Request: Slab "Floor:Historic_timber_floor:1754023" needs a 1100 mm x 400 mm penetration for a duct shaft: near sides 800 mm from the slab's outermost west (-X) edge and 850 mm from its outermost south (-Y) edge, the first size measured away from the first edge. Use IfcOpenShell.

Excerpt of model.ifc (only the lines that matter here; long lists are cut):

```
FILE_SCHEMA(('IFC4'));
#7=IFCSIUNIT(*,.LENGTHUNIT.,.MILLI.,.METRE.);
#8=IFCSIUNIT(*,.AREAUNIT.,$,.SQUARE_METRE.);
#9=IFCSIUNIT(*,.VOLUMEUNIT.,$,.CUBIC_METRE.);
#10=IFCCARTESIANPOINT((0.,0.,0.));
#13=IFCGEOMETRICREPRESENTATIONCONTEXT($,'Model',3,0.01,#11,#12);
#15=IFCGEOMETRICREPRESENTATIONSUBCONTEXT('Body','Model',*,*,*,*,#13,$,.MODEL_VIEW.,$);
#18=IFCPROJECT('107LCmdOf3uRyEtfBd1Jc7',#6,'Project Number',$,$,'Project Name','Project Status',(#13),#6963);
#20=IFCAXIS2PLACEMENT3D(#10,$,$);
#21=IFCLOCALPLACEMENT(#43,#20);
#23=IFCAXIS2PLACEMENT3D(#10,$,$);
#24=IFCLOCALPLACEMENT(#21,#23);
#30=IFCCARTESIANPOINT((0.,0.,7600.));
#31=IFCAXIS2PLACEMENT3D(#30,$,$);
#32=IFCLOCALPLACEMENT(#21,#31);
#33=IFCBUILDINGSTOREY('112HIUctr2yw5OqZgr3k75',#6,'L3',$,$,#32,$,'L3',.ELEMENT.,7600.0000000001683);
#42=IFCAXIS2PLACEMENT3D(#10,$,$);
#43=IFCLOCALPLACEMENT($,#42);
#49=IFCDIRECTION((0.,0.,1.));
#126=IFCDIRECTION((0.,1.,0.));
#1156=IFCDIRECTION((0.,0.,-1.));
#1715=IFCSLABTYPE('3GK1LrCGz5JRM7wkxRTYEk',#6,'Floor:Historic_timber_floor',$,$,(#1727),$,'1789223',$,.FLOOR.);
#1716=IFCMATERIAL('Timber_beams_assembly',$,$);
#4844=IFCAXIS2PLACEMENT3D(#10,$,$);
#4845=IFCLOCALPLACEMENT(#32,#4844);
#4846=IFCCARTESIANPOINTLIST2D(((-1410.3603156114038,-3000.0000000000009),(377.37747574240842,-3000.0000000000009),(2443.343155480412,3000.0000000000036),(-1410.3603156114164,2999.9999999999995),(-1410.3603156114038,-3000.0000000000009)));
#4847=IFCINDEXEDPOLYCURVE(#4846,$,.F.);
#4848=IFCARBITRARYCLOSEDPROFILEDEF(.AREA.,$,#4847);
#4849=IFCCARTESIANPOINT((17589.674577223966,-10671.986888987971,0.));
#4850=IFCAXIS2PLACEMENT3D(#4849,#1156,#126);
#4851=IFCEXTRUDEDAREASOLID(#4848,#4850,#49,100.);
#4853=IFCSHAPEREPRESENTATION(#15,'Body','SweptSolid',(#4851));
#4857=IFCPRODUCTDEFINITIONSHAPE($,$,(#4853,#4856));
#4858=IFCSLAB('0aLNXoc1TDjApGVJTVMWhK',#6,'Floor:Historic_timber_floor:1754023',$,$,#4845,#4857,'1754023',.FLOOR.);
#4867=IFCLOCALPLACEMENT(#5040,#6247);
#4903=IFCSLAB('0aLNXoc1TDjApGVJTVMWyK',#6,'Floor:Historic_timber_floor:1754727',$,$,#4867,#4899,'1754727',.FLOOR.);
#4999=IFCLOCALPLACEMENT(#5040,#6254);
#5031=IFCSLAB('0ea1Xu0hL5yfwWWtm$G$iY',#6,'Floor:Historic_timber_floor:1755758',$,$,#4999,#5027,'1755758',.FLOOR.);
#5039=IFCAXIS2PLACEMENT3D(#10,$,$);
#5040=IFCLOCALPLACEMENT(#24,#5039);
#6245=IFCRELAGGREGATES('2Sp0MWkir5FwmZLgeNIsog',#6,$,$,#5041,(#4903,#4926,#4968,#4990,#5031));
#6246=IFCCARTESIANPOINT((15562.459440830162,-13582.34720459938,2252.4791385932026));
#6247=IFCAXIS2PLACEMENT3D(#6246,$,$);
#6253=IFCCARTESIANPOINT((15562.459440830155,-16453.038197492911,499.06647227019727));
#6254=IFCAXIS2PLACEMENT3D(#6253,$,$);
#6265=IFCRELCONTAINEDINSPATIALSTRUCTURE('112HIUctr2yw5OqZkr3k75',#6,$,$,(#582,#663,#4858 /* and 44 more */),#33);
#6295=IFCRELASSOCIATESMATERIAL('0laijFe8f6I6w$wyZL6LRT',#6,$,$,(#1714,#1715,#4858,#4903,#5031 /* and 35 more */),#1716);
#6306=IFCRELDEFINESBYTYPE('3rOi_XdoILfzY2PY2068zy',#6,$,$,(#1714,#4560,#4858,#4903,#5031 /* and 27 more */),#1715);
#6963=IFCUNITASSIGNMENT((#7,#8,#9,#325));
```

```python
import numpy as np
import ifcopenshell
import ifcopenshell.api.feature
import ifcopenshell.api.geometry
import ifcopenshell.api.root
import ifcopenshell.geom
import ifcopenshell.util.placement
import ifcopenshell.util.representation
import ifcopenshell.util.shape
import ifcopenshell.util.unit

model = ifcopenshell.open("model.ifc")
unit_scale = ifcopenshell.util.unit.calculate_unit_scale(model)
settings = ifcopenshell.geom.settings()


def volume(element):
    """Net volume in cubic metres, openings subtracted."""
    shape = ifcopenshell.geom.create_shape(settings, element)
    return ifcopenshell.util.shape.get_volume(shape.geometry)


slab = model.by_id(4858)
before = volume(slab)

# Extent in the slab's own axes, in metres. The edges named are its -X and -Y sides.
slab_shape = ifcopenshell.geom.create_shape(settings, slab)
vertices = ifcopenshell.util.shape.get_vertices(slab_shape.geometry)
x_min, y_min, bottom = vertices.min(axis=0)
top = vertices[:, 2].max()

opening = ifcopenshell.api.root.create_entity(model, ifc_class="IfcOpeningElement", name="Duct shaft opening", predefined_type="OPENING")
context = ifcopenshell.util.representation.get_context(model, "Model", "Body", "MODEL_VIEW")
width, depth = 1.1, 0.4
outline = [(0.0, 0.0), (width, 0.0), (width, depth), (0.0, depth), (0.0, 0.0)]
# Overshoot both faces by 50 mm so the cut is clean.
shape = ifcopenshell.api.geometry.add_slab_representation(
    model, context=context, depth=top - bottom + 0.1, polyline=outline
)
ifcopenshell.api.geometry.assign_representation(model, product=opening, representation=shape)

matrix = ifcopenshell.util.placement.get_local_placement(slab.ObjectPlacement)
matrix[:, 3] = matrix @ np.append(np.array([x_min + 0.8, y_min + 0.85, bottom - 0.05]) / unit_scale, 1.0)
ifcopenshell.api.geometry.edit_object_placement(model, product=opening, matrix=matrix, is_si=False)
ifcopenshell.api.feature.add_feature(model, feature=opening, element=slab)

after = volume(slab)

print(f"slab volume {before:.3f} -> {after:.3f} m3")

model.write("model_updated.ifc")
```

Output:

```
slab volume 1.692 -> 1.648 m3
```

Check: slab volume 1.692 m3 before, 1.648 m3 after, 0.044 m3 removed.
